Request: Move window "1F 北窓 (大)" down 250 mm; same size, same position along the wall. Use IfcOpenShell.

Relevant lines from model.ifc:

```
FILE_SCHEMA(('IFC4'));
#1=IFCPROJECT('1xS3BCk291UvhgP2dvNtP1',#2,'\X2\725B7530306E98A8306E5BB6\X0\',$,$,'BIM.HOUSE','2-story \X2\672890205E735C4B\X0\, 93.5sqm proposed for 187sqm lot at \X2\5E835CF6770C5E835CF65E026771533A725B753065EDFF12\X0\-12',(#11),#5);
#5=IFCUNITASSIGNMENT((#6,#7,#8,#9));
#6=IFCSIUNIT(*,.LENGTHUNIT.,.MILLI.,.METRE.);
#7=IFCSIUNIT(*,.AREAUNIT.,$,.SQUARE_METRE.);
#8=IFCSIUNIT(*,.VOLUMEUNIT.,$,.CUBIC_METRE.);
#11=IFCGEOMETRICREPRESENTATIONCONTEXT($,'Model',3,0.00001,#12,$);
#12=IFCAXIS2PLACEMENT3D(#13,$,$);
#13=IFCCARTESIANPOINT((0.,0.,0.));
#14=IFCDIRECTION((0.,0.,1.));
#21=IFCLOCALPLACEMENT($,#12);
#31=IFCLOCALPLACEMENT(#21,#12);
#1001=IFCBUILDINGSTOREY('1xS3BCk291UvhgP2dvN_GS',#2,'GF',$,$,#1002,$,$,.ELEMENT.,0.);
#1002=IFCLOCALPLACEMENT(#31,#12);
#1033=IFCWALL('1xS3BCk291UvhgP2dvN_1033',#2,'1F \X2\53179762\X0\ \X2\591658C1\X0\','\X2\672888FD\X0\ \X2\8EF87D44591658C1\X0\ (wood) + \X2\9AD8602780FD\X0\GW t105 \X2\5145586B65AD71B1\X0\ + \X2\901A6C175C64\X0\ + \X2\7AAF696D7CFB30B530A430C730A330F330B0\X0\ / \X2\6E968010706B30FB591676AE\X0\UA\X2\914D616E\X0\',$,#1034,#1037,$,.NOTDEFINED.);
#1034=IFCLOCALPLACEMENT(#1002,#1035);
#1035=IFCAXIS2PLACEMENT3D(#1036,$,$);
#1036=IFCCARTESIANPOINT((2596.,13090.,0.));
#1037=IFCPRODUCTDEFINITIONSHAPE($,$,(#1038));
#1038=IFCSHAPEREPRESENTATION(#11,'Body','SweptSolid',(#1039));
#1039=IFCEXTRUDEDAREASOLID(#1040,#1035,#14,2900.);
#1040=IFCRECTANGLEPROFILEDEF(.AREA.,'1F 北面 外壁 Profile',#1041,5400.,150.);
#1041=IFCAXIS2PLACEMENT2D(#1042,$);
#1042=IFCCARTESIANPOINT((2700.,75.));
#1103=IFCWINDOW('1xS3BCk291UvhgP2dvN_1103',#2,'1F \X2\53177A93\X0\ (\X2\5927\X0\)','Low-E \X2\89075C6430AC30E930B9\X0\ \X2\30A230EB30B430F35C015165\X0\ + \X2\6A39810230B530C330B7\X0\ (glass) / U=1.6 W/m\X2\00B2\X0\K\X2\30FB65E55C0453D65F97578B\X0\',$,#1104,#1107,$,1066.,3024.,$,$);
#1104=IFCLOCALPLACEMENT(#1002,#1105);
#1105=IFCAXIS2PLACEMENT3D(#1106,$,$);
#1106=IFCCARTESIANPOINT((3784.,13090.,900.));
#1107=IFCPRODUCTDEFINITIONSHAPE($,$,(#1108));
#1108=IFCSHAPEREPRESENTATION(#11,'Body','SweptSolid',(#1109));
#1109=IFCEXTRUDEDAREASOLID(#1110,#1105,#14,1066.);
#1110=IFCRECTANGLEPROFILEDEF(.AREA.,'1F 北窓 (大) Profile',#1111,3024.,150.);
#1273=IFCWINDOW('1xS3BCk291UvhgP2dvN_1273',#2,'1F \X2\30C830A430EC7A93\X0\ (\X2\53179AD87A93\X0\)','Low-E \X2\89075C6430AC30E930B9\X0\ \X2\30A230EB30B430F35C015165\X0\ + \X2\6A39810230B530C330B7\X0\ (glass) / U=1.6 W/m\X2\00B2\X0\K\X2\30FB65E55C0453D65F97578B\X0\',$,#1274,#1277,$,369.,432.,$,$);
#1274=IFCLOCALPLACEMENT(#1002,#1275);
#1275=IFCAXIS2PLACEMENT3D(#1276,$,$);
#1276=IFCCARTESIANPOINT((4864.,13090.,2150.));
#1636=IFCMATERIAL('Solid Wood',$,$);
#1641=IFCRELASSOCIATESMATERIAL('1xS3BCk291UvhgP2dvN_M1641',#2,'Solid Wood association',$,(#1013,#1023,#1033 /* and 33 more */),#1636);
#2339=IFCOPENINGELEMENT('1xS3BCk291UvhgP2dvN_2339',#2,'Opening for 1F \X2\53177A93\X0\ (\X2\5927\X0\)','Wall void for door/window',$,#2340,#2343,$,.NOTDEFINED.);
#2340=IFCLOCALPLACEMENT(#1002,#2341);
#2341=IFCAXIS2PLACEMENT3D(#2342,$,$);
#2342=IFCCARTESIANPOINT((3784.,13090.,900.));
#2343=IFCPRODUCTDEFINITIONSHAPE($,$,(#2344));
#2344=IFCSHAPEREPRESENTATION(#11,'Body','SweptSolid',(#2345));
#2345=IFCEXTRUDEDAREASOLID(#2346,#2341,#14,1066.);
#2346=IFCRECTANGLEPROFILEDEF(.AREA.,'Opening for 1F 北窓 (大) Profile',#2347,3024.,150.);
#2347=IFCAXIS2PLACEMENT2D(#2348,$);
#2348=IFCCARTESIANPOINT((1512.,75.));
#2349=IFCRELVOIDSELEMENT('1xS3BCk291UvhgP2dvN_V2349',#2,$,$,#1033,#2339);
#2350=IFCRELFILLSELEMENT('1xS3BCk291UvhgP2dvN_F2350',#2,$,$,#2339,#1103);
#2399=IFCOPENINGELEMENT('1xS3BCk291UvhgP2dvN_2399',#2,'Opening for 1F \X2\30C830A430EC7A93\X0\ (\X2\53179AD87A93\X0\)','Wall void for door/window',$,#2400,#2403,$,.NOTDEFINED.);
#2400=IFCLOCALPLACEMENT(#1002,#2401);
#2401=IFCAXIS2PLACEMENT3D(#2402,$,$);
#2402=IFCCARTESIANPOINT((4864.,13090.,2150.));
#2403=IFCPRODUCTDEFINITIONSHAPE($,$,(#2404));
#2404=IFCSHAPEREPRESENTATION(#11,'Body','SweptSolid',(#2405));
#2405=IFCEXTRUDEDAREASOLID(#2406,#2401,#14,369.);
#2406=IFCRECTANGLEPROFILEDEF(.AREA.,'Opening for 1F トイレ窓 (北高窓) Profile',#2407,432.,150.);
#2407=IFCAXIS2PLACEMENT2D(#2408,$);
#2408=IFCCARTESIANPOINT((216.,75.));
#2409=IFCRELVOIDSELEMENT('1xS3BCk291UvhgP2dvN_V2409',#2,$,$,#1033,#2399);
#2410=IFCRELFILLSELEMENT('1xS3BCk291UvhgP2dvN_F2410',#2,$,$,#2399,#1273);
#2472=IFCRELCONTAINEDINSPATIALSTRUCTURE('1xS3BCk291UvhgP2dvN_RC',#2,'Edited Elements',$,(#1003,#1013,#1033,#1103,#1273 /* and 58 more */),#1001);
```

```python
import numpy as np
import ifcopenshell
import ifcopenshell.api.geometry
import ifcopenshell.util.placement
import ifcopenshell.util.unit

model = ifcopenshell.open("model.ifc")
unit_scale = ifcopenshell.util.unit.calculate_unit_scale(model)

window = model.by_id(1103)
opening = window.FillsVoids[0].RelatingOpeningElement
dz = -0.25 / unit_scale

shift = np.array([0.0, 0.0, dz])
# The window is not placed relative to its opening, so move both.
for product in (opening, window):
    matrix = ifcopenshell.util.placement.get_local_placement(product.ObjectPlacement)
    matrix[:3, 3] += shift
    ifcopenshell.api.geometry.edit_object_placement(model, product=product, matrix=matrix, is_si=False)

print(f"moved by {dz * unit_scale:+.3f} m")

model.write("model_rev.ifc")
```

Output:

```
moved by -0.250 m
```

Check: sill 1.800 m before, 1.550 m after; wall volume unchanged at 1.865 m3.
